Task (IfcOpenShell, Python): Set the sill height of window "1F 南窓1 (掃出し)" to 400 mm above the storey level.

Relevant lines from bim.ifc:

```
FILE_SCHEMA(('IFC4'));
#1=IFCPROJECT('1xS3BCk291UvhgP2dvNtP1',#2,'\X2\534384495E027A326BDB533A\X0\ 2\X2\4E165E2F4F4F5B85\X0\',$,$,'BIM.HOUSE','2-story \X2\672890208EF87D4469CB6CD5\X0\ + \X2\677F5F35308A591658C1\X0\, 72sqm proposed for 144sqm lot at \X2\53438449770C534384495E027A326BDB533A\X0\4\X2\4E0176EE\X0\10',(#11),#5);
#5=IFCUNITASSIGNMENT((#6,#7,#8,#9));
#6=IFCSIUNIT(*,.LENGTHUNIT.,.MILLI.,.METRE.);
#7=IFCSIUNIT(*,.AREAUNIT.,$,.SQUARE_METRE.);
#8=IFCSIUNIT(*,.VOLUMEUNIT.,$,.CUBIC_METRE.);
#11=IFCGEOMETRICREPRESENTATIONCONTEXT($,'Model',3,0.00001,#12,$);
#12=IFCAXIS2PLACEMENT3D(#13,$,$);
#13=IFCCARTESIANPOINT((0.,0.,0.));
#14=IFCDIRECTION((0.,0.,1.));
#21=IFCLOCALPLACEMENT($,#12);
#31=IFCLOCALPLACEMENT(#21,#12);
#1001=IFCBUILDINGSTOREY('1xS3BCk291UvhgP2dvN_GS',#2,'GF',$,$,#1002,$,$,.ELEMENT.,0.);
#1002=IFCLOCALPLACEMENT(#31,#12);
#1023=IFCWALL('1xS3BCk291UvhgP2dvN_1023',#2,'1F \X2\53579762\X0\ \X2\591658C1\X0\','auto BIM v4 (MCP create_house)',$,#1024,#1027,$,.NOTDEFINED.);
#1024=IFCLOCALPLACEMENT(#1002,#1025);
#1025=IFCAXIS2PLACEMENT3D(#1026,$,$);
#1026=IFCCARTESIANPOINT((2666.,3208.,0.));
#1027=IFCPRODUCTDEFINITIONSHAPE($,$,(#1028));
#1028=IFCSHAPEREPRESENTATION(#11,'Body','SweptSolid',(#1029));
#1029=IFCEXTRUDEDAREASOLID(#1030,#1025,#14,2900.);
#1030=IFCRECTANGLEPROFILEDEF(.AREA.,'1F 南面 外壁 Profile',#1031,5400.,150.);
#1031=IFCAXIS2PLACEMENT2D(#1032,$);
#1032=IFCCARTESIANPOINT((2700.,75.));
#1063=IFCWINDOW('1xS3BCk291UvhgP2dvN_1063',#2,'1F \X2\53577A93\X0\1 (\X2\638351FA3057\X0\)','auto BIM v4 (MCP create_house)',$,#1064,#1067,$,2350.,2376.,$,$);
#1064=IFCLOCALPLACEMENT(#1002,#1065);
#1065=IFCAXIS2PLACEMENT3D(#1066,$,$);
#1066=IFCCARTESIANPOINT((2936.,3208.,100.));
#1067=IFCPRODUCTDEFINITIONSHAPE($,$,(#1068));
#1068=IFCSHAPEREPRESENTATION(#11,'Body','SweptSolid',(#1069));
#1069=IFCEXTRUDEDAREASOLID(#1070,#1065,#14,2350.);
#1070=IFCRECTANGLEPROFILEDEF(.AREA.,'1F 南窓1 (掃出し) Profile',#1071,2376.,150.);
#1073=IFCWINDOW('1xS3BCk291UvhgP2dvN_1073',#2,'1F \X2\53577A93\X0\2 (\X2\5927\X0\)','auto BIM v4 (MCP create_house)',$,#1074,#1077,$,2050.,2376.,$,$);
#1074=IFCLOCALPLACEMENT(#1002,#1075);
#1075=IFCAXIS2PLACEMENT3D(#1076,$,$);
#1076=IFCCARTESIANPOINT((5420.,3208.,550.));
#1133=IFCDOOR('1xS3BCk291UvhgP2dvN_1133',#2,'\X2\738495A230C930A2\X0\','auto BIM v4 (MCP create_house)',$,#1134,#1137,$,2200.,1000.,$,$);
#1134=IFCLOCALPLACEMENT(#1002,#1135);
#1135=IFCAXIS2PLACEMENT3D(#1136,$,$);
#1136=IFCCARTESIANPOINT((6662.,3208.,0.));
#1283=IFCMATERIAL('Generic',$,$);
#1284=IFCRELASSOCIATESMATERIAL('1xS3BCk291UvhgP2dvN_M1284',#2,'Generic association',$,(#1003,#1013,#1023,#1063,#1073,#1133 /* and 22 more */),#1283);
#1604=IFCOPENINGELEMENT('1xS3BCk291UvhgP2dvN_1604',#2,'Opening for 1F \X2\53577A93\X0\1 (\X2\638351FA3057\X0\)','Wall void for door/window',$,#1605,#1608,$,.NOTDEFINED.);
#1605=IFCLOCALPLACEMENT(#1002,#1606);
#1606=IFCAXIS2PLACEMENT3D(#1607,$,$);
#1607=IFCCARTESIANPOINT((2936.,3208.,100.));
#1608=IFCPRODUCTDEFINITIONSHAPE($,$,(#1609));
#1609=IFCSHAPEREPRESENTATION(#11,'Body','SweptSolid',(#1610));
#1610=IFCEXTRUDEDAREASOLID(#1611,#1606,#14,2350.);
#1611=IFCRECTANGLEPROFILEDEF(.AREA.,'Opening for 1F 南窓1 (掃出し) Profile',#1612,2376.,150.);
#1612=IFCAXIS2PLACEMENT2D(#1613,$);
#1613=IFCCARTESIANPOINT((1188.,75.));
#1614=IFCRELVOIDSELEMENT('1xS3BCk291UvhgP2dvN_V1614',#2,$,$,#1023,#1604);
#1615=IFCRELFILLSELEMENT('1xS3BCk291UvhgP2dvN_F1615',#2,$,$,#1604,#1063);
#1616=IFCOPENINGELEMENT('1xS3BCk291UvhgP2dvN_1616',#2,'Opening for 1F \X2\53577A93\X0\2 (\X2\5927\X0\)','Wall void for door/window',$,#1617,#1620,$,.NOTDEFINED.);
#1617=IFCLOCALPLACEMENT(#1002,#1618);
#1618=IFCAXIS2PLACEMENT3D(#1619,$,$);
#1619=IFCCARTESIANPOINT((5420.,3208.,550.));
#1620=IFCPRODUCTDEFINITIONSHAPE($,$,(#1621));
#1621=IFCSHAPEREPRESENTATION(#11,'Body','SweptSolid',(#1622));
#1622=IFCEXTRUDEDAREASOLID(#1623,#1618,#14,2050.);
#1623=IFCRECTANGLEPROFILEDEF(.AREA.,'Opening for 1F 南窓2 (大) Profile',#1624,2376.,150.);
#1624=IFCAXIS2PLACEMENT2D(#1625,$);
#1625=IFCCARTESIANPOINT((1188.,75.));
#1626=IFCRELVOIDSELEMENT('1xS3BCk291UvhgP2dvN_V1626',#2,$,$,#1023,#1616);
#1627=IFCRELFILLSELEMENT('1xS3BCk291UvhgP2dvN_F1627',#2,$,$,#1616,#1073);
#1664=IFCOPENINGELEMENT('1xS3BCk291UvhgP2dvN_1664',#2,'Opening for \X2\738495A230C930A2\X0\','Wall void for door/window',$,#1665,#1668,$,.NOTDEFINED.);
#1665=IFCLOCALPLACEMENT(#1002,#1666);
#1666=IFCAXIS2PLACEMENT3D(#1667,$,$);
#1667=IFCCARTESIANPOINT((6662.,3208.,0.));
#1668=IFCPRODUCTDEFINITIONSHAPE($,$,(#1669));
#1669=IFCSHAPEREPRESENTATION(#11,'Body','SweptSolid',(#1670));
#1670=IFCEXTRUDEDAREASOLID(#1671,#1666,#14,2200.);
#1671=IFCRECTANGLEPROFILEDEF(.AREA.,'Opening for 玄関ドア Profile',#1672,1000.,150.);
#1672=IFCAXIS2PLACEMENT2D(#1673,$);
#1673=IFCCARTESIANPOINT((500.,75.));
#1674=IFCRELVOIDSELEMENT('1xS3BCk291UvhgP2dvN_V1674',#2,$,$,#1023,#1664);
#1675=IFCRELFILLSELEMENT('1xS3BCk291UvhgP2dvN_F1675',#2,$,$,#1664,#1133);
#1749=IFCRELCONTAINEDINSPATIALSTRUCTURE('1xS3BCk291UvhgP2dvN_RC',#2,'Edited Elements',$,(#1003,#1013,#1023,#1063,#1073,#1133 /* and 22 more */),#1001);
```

```python
import numpy as np
import ifcopenshell
import ifcopenshell.api.geometry
import ifcopenshell.geom
import ifcopenshell.util.element
import ifcopenshell.util.placement
import ifcopenshell.util.shape
import ifcopenshell.util.unit

model = ifcopenshell.open("bim.ifc")
unit_scale = ifcopenshell.util.unit.calculate_unit_scale(model)

window = model.by_guid("1xS3BCk291UvhgP2dvN_1063")
opening = window.FillsVoids[0].RelatingOpeningElement
storey = ifcopenshell.util.element.get_container(window, ifc_class="IfcBuildingStorey")
level = ifcopenshell.util.placement.get_local_placement(storey.ObjectPlacement)[2, 3]

# The opening's origin need not be at the sill, so measure its lowest point.
shape = ifcopenshell.geom.create_shape(ifcopenshell.geom.settings(), opening)
bottom = ifcopenshell.util.shape.get_shape_bottom_elevation(shape, shape.geometry) / unit_scale
dz = level + 0.4 / unit_scale - bottom

shift = np.array([0.0, 0.0, dz])
# The window is not placed relative to its opening, so move both.
for product in (opening, window):
    matrix = ifcopenshell.util.placement.get_local_placement(product.ObjectPlacement)
    matrix[:3, 3] += shift
    ifcopenshell.api.geometry.edit_object_placement(model, product=product, matrix=matrix, is_si=False)

print(f"moved by {dz * unit_scale:+.3f} m")

model.write("bim_edited.ifc")
```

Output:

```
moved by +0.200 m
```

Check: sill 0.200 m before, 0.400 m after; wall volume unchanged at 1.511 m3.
